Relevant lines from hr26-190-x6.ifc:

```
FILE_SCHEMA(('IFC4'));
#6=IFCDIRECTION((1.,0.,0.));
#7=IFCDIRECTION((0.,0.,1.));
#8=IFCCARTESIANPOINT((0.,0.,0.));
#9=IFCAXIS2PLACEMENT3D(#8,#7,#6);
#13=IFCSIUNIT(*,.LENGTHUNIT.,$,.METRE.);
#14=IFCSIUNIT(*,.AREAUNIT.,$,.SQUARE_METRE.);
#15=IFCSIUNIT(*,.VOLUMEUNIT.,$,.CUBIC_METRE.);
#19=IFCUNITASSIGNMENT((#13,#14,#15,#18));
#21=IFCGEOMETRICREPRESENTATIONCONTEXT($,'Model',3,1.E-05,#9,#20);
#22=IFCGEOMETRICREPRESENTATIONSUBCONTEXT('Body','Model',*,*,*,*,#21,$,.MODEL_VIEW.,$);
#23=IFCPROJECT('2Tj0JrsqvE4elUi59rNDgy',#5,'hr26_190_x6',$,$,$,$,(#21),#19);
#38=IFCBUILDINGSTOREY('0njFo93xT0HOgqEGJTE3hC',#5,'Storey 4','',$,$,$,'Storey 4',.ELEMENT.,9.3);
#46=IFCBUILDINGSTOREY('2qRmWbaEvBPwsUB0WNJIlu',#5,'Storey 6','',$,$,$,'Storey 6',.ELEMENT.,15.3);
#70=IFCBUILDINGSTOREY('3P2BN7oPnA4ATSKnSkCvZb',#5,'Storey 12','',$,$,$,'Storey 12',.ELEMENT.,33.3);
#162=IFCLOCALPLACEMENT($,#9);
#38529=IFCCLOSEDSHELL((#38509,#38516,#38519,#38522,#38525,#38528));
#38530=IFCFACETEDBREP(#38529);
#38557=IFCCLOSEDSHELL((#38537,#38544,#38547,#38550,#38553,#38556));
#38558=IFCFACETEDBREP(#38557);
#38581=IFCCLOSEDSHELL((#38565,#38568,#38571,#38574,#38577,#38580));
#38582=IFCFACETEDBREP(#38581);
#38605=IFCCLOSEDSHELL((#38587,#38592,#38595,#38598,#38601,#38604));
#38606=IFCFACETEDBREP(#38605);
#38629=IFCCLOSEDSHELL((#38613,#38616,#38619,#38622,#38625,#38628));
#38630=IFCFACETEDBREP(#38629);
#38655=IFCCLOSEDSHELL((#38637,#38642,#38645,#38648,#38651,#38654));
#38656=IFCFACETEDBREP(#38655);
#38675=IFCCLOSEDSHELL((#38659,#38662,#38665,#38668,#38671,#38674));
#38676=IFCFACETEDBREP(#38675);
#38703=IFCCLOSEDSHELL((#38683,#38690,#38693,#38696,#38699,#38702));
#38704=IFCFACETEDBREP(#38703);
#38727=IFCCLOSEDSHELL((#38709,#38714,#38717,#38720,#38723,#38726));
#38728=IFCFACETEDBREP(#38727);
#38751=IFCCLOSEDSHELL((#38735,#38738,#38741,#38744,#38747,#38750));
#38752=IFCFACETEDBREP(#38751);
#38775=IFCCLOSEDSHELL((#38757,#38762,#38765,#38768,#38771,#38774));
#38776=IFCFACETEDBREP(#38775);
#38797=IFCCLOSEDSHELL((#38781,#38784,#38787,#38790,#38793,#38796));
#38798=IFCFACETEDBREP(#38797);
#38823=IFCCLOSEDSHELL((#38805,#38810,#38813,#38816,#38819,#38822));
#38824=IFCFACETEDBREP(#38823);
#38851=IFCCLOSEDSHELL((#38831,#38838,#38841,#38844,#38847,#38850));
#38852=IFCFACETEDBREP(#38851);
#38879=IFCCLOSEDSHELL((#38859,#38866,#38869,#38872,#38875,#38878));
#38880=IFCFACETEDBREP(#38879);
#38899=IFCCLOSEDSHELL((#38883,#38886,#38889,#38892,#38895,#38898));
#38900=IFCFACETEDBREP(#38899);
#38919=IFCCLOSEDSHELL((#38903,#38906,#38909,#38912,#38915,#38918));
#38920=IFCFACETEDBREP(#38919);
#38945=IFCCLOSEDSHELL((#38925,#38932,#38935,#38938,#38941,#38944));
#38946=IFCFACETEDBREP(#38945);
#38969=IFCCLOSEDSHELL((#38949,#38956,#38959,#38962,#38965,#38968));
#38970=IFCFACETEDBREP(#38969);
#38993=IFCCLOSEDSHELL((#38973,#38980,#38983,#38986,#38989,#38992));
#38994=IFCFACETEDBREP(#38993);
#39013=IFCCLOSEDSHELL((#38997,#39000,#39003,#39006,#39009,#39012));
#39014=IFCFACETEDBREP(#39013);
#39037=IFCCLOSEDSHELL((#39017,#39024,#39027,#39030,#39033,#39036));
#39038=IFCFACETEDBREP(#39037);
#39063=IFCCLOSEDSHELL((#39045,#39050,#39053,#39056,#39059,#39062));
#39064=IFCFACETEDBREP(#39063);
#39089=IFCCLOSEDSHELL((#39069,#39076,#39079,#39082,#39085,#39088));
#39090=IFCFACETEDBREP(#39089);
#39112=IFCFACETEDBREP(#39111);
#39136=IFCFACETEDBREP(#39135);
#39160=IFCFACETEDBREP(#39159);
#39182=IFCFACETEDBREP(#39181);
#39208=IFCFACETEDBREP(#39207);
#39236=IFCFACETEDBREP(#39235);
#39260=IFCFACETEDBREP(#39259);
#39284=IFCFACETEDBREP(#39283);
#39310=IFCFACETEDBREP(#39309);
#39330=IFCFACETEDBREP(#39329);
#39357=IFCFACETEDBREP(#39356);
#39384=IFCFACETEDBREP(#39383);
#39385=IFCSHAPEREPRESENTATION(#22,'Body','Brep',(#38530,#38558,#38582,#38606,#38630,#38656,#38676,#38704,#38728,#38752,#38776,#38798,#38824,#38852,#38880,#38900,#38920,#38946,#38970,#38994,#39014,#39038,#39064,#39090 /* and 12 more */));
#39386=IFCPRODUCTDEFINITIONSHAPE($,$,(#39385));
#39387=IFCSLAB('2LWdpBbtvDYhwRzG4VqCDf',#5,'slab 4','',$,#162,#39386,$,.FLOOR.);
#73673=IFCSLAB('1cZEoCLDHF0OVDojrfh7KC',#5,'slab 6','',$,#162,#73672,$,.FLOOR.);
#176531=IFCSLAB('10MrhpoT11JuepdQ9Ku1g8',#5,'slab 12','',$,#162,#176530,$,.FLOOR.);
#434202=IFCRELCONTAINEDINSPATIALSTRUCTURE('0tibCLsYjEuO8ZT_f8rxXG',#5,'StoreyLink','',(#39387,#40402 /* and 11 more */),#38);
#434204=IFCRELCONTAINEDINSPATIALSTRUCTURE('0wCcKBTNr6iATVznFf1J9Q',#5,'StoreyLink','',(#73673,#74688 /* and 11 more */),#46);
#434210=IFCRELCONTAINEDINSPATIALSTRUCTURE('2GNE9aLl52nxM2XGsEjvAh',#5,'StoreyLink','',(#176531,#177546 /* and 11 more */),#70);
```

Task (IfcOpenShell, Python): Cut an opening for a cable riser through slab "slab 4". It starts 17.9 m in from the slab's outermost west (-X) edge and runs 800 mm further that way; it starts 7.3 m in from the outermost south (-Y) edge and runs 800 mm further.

```python
import numpy as np
import ifcopenshell
import ifcopenshell.api.feature
import ifcopenshell.api.geometry
import ifcopenshell.api.root
import ifcopenshell.geom
import ifcopenshell.util.placement
import ifcopenshell.util.representation
import ifcopenshell.util.shape
import ifcopenshell.util.unit

model = ifcopenshell.open("hr26-190-x6.ifc")
unit_scale = ifcopenshell.util.unit.calculate_unit_scale(model)
settings = ifcopenshell.geom.settings()


def volume(element):
    """Net volume in cubic metres, openings subtracted."""
    shape = ifcopenshell.geom.create_shape(settings, element)
    return ifcopenshell.util.shape.get_volume(shape.geometry)


slab = model.by_id(39387)
before = volume(slab)

# Extent in the slab's own axes, in metres. The edges named are its -X and -Y sides.
slab_shape = ifcopenshell.geom.create_shape(settings, slab)
vertices = ifcopenshell.util.shape.get_vertices(slab_shape.geometry)
x_min, y_min, bottom = vertices.min(axis=0)
top = vertices[:, 2].max()

opening = ifcopenshell.api.root.create_entity(model, ifc_class="IfcOpeningElement", name="Cable riser opening", predefined_type="OPENING")
context = ifcopenshell.util.representation.get_context(model, "Model", "Body", "MODEL_VIEW")
width, depth = 0.8, 0.8
outline = [(0.0, 0.0), (width, 0.0), (width, depth), (0.0, depth), (0.0, 0.0)]
# Overshoot both faces by 50 mm so the cut is clean.
shape = ifcopenshell.api.geometry.add_slab_representation(
    model, context=context, depth=top - bottom + 0.1, polyline=outline
)
ifcopenshell.api.geometry.assign_representation(model, product=opening, representation=shape)

matrix = ifcopenshell.util.placement.get_local_placement(slab.ObjectPlacement)
matrix[:, 3] = matrix @ np.append(np.array([x_min + 17.9, y_min + 7.3, bottom - 0.05]) / unit_scale, 1.0)
ifcopenshell.api.geometry.edit_object_placement(model, product=opening, matrix=matrix, is_si=False)
ifcopenshell.api.feature.add_feature(model, feature=opening, element=slab)

after = volume(slab)

print(f"slab volume {before:.3f} -> {after:.3f} m3")

model.write("hr26-190-x6-out.ifc")
```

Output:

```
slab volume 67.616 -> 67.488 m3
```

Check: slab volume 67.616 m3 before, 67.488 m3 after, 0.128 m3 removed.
